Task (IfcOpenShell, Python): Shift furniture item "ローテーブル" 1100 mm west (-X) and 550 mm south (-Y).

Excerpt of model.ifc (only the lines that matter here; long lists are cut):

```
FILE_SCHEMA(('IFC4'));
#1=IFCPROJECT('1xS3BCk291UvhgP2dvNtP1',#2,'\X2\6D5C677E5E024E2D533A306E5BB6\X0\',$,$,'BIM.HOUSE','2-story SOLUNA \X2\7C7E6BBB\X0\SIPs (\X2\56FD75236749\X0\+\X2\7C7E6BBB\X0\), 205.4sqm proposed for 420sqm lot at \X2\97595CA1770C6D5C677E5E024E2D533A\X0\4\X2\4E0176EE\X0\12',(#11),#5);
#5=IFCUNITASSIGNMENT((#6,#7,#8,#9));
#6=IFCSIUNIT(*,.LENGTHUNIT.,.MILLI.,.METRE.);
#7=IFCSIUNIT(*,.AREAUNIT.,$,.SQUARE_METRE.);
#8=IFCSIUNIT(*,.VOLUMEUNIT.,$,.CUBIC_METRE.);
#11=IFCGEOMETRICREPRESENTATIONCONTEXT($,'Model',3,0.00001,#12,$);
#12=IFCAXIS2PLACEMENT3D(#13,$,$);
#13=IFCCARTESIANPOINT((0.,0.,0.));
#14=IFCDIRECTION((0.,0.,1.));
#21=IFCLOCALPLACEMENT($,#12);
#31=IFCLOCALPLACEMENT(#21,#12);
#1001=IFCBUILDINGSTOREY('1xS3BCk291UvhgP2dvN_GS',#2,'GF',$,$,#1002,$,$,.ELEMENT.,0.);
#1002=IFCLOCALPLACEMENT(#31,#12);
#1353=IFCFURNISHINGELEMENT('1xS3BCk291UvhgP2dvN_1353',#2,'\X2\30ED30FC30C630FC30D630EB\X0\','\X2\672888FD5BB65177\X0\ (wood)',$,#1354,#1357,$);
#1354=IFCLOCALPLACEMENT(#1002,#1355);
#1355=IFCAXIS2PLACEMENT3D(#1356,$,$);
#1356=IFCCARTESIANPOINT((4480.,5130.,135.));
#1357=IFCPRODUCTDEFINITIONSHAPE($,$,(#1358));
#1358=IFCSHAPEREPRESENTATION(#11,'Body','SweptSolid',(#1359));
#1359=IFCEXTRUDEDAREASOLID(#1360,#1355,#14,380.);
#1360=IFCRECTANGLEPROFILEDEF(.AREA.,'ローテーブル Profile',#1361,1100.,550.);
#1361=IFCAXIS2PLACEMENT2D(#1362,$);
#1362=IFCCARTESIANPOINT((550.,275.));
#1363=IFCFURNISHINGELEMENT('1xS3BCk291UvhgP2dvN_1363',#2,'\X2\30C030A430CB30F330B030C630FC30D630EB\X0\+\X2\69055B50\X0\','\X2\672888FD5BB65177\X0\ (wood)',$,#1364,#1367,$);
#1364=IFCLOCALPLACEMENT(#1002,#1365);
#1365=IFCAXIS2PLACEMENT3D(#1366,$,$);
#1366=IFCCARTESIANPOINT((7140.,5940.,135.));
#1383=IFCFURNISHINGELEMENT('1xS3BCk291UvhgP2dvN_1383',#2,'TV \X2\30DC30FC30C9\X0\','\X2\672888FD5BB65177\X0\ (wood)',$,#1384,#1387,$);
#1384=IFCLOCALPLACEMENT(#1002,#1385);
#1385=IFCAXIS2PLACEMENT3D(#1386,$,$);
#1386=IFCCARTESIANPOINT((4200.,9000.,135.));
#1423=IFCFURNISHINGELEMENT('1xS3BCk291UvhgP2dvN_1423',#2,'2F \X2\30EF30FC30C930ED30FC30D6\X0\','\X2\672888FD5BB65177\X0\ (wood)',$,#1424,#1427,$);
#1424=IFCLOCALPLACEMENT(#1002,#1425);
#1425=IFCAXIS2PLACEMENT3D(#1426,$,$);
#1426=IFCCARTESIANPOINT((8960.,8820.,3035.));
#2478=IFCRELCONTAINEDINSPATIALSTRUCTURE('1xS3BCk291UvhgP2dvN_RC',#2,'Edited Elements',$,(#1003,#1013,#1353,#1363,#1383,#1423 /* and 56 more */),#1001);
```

```python
import ifcopenshell
import ifcopenshell.api.geometry
import ifcopenshell.util.placement

model = ifcopenshell.open("model.ifc")

item = model.by_id(1353)
matrix = ifcopenshell.util.placement.get_local_placement(item.ObjectPlacement)
matrix[0, 3] -= 1100.0
matrix[1, 3] -= 550.0
ifcopenshell.api.geometry.edit_object_placement(model, product=item, matrix=matrix, is_si=False)

print(ifcopenshell.util.placement.get_local_placement(item.ObjectPlacement).round(3) + 0.0)

model.write("model_rev.ifc")
```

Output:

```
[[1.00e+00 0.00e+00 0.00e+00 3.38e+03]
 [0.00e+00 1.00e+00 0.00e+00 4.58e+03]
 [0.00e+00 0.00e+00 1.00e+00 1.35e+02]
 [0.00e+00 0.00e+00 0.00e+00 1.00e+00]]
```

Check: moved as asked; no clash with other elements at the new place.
